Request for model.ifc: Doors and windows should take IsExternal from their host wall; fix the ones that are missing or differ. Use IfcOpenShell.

First a look at what the model holds.

```python
import ifcopenshell
import ifcopenshell.util.element

model = ifcopenshell.open("model.ifc")
print(model.schema)
seen = {}
for e in model.by_type("IfcDoor") + model.by_type("IfcWindow"):
    if not e.FillsVoids:
        continue
    host = e.FillsVoids[0].RelatingOpeningElement.VoidsElements[0].RelatingBuildingElement
    own = ifcopenshell.util.element.get_pset(e, f"Pset_{e.is_a()[3:].removesuffix('StandardCase')}Common", "IsExternal")
    wall = ifcopenshell.util.element.get_pset(host, "Pset_WallCommon", "IsExternal")
    seen[e.is_a(), own, wall] = seen.get((e.is_a(), own, wall), 0) + 1
for (cls, own, wall), count in sorted(seen.items(), key=str):
    print(count, cls, "IsExternal:", own, "| host wall:", wall)
```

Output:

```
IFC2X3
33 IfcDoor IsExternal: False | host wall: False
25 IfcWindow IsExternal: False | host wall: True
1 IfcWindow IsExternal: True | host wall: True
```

```python
import ifcopenshell
import ifcopenshell.api.pset
import ifcopenshell.util.element

model = ifcopenshell.open("model.ifc")

count = 0
for ifc_class, pset_name in (("IfcDoor", "Pset_DoorCommon"), ("IfcWindow", "Pset_WindowCommon")):
    for e in model.by_type(ifc_class):
        if not e.FillsVoids:
            continue
        host = e.FillsVoids[0].RelatingOpeningElement.VoidsElements[0].RelatingBuildingElement
        external = ifcopenshell.util.element.get_pset(host, "Pset_WallCommon", "IsExternal")
        if external is None or ifcopenshell.util.element.get_pset(e, pset_name, "IsExternal") == external:
            continue
        pset = ifcopenshell.api.pset.add_pset(model, product=e, name=pset_name)
        ifcopenshell.api.pset.edit_pset(model, pset=pset, properties={"IsExternal": external})
        count += 1

print(count, "updated")

model.write("model_rev.ifc")
```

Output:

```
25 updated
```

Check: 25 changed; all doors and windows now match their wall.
